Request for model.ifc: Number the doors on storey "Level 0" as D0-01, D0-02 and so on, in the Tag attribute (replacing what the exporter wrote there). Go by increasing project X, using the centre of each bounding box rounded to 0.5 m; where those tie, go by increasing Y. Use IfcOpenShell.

First a look at what the model holds.

```python
import ifcopenshell
import ifcopenshell.util.element
import ifcopenshell.util.placement

model = ifcopenshell.open("model.ifc")
print(model.schema)
storey = next(s for s in model.by_type("IfcBuildingStorey") if s.Name == "Level 0")
doors = [e for e in ifcopenshell.util.element.get_decomposition(storey) if e.is_a("IfcDoor")]
for e in sorted(doors, key=lambda e: e.id()):
    origin = ifcopenshell.util.placement.get_local_placement(e.ObjectPlacement)[:3, 3]
    print(e.id(), e.Tag, e.Name, origin.round(2) + 0.0, sep=" | ")
```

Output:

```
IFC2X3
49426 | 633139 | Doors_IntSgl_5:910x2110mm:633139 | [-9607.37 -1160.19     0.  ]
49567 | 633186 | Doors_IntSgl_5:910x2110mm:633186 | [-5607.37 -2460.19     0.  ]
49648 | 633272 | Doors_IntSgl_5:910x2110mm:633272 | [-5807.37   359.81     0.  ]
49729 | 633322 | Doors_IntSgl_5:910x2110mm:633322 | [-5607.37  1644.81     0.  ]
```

```python
import ifcopenshell
import ifcopenshell.geom
import ifcopenshell.util.element
import ifcopenshell.util.shape

model = ifcopenshell.open("model.ifc")
settings = ifcopenshell.geom.settings()
settings.set("use-world-coords", True)


def centre(element):
    shape = ifcopenshell.geom.create_shape(settings, element)
    return ifcopenshell.util.shape.get_bbox_centroid(shape.geometry)


storey = next(s for s in model.by_type("IfcBuildingStorey") if s.Name == "Level 0")
doors = [e for e in ifcopenshell.util.element.get_decomposition(storey) if e.is_a("IfcDoor")]

# Insertion points can sit at a corner or the storey origin, so sort by the geometry (in metres).
centres = {e: centre(e) for e in doors}
doors.sort(key=lambda e: (round(centres[e][0] / 0.5), centres[e][1]))

for i, e in enumerate(doors, start=1):
    number = f"D0-{i:02d}"
    e.Tag = number
    print(e.id(), number)

model.write("model_v2.ifc")
```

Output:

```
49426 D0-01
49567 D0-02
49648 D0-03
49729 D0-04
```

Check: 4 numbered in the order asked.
